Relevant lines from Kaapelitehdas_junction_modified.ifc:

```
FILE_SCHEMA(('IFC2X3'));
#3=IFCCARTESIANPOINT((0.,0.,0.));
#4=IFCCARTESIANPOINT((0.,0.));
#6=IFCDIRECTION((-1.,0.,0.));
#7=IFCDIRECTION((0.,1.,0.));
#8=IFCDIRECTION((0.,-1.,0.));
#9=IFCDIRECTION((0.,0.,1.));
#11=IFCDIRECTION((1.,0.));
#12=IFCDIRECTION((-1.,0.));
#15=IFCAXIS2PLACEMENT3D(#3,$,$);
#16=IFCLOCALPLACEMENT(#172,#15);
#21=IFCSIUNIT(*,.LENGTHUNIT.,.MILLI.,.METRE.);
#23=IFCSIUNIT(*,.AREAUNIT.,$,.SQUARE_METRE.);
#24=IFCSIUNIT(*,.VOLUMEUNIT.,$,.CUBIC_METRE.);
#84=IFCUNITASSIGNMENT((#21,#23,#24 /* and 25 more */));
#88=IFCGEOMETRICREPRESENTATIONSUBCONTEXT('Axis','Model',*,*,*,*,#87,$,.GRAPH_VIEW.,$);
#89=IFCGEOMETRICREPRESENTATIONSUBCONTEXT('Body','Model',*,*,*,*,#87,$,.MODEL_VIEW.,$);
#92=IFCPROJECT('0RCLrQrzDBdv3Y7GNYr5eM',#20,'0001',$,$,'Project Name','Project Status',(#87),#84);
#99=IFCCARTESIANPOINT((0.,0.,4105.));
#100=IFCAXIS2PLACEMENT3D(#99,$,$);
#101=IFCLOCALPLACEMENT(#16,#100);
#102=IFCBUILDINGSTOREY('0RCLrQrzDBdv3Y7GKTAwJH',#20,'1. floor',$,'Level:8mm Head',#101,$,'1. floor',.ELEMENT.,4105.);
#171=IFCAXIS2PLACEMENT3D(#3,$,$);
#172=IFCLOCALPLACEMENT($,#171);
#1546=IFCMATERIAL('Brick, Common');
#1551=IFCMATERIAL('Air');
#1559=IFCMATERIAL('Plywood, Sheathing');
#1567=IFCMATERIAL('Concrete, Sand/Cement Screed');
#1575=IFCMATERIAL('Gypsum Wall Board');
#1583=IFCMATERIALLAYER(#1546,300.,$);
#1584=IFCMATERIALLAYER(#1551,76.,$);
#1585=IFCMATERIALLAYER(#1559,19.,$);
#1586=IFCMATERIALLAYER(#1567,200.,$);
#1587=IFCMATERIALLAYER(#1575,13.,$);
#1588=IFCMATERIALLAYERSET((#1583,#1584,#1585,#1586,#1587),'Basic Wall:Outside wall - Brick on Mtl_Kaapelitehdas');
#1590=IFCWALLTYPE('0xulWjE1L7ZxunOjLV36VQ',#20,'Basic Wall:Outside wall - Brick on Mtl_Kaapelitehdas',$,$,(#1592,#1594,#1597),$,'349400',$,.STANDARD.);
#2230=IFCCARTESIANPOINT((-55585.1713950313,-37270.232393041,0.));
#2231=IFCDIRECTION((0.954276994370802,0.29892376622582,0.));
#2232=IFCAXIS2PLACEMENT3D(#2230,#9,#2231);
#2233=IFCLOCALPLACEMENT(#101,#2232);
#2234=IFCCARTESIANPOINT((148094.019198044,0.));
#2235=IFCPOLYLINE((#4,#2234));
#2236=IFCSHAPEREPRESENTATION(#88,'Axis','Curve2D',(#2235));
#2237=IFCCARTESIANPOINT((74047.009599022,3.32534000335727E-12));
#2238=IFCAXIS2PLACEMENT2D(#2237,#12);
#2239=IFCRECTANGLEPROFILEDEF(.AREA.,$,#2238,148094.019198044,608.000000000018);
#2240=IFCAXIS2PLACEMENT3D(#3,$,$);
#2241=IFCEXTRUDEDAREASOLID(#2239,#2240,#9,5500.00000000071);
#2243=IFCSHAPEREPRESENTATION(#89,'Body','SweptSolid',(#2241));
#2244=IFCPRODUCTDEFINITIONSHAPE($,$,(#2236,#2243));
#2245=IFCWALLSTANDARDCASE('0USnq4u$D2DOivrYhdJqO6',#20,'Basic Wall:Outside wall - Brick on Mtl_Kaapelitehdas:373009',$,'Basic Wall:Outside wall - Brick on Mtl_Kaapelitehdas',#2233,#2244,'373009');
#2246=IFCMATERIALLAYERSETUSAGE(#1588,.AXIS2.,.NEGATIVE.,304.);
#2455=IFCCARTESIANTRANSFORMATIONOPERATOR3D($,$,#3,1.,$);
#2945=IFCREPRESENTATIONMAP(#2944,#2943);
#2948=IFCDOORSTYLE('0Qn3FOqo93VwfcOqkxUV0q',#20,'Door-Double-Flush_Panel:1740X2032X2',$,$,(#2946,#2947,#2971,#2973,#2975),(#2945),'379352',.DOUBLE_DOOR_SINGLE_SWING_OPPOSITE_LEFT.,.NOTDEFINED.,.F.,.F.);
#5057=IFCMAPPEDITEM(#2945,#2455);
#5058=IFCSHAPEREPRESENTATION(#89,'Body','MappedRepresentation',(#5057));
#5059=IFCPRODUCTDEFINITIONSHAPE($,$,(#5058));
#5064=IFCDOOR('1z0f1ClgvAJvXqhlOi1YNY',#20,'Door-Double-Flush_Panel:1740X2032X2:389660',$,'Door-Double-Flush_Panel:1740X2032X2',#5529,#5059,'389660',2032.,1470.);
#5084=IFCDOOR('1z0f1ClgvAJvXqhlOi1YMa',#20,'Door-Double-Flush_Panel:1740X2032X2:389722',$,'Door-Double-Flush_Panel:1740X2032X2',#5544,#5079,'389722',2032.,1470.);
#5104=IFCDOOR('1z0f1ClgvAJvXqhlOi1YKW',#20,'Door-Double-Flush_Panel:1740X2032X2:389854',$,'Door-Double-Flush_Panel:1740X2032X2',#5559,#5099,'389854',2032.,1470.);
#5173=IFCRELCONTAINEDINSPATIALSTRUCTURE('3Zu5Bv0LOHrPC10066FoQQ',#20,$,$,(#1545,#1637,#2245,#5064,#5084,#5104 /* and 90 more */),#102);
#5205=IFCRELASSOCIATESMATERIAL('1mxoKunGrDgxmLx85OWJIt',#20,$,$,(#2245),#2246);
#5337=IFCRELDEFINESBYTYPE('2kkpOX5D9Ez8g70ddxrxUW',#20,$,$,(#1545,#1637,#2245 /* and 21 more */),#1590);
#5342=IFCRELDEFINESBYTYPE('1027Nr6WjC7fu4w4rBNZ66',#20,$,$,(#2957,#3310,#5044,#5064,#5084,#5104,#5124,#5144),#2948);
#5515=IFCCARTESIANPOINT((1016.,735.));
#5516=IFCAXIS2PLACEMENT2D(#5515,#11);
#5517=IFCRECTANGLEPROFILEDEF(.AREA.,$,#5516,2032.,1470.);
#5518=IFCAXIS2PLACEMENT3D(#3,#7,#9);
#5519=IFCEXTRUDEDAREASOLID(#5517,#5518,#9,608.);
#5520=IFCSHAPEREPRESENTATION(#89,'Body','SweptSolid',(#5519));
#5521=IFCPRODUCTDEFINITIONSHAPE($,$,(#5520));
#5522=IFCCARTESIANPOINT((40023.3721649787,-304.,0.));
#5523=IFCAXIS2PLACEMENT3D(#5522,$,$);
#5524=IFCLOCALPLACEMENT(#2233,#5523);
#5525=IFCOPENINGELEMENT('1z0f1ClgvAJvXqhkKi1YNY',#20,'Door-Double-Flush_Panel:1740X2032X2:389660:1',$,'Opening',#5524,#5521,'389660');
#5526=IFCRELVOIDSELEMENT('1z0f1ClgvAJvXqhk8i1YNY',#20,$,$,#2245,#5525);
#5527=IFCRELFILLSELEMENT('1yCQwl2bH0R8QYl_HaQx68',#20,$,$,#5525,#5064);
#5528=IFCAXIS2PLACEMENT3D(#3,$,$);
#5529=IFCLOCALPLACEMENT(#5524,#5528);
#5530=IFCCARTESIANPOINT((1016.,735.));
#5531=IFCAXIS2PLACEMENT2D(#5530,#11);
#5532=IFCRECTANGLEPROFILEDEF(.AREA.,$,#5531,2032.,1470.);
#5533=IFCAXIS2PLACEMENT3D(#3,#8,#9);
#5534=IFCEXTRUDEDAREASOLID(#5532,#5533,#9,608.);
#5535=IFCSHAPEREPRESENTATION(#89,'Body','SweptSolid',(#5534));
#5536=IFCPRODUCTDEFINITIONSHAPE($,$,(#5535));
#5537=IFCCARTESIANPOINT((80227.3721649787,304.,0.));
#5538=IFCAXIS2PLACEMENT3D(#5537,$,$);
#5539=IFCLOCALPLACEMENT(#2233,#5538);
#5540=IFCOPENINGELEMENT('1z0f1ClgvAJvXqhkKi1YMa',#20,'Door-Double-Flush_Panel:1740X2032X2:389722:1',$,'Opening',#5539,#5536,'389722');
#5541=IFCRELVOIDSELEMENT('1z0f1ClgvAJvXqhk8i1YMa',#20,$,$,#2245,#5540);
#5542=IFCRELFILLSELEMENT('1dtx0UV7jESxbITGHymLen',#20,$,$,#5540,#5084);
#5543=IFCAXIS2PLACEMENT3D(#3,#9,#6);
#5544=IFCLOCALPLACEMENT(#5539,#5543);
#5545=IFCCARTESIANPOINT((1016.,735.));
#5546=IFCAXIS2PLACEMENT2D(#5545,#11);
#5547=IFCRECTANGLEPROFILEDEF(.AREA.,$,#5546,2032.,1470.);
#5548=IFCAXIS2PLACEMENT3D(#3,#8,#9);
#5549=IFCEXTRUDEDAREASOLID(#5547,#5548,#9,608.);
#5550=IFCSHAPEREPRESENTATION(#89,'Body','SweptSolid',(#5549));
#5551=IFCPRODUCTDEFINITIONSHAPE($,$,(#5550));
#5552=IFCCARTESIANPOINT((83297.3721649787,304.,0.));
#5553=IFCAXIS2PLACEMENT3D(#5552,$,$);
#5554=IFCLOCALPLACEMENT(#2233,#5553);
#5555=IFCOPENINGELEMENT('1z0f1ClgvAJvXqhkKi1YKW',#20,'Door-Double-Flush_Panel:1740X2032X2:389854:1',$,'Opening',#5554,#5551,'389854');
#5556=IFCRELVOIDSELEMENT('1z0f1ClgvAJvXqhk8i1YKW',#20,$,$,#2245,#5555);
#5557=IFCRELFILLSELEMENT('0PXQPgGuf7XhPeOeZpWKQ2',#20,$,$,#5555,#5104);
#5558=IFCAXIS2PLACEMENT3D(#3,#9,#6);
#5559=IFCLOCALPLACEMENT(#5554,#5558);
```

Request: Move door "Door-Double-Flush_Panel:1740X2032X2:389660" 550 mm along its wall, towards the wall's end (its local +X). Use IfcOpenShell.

```python
import ifcopenshell
import ifcopenshell.api.geometry
import ifcopenshell.util.placement

model = ifcopenshell.open("Kaapelitehdas_junction_modified.ifc")

door = model.by_guid("1z0f1ClgvAJvXqhlOi1YNY")
opening = door.FillsVoids[0].RelatingOpeningElement
wall = opening.VoidsElements[0].RelatingBuildingElement

wall_matrix = ifcopenshell.util.placement.get_local_placement(wall.ObjectPlacement)
shift = wall_matrix[:3, 0] * 550.0
before = ifcopenshell.util.placement.get_local_placement(door.ObjectPlacement)[:3, 3].copy()

# The door is placed relative to its opening, so it follows when the opening moves.
matrix = ifcopenshell.util.placement.get_local_placement(opening.ObjectPlacement)
matrix[:3, 3] += shift
ifcopenshell.api.geometry.edit_object_placement(
    model, product=opening, matrix=matrix, is_si=False, should_transform_children=True
)

after = ifcopenshell.util.placement.get_local_placement(door.ObjectPlacement)[:3, 3]
print("door moved by", (after - before).round(3) + 0.0)

model.write("Kaapelitehdas_junction_modified_edited.ifc")
```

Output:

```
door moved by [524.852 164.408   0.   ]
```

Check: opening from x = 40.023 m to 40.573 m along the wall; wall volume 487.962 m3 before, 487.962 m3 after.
